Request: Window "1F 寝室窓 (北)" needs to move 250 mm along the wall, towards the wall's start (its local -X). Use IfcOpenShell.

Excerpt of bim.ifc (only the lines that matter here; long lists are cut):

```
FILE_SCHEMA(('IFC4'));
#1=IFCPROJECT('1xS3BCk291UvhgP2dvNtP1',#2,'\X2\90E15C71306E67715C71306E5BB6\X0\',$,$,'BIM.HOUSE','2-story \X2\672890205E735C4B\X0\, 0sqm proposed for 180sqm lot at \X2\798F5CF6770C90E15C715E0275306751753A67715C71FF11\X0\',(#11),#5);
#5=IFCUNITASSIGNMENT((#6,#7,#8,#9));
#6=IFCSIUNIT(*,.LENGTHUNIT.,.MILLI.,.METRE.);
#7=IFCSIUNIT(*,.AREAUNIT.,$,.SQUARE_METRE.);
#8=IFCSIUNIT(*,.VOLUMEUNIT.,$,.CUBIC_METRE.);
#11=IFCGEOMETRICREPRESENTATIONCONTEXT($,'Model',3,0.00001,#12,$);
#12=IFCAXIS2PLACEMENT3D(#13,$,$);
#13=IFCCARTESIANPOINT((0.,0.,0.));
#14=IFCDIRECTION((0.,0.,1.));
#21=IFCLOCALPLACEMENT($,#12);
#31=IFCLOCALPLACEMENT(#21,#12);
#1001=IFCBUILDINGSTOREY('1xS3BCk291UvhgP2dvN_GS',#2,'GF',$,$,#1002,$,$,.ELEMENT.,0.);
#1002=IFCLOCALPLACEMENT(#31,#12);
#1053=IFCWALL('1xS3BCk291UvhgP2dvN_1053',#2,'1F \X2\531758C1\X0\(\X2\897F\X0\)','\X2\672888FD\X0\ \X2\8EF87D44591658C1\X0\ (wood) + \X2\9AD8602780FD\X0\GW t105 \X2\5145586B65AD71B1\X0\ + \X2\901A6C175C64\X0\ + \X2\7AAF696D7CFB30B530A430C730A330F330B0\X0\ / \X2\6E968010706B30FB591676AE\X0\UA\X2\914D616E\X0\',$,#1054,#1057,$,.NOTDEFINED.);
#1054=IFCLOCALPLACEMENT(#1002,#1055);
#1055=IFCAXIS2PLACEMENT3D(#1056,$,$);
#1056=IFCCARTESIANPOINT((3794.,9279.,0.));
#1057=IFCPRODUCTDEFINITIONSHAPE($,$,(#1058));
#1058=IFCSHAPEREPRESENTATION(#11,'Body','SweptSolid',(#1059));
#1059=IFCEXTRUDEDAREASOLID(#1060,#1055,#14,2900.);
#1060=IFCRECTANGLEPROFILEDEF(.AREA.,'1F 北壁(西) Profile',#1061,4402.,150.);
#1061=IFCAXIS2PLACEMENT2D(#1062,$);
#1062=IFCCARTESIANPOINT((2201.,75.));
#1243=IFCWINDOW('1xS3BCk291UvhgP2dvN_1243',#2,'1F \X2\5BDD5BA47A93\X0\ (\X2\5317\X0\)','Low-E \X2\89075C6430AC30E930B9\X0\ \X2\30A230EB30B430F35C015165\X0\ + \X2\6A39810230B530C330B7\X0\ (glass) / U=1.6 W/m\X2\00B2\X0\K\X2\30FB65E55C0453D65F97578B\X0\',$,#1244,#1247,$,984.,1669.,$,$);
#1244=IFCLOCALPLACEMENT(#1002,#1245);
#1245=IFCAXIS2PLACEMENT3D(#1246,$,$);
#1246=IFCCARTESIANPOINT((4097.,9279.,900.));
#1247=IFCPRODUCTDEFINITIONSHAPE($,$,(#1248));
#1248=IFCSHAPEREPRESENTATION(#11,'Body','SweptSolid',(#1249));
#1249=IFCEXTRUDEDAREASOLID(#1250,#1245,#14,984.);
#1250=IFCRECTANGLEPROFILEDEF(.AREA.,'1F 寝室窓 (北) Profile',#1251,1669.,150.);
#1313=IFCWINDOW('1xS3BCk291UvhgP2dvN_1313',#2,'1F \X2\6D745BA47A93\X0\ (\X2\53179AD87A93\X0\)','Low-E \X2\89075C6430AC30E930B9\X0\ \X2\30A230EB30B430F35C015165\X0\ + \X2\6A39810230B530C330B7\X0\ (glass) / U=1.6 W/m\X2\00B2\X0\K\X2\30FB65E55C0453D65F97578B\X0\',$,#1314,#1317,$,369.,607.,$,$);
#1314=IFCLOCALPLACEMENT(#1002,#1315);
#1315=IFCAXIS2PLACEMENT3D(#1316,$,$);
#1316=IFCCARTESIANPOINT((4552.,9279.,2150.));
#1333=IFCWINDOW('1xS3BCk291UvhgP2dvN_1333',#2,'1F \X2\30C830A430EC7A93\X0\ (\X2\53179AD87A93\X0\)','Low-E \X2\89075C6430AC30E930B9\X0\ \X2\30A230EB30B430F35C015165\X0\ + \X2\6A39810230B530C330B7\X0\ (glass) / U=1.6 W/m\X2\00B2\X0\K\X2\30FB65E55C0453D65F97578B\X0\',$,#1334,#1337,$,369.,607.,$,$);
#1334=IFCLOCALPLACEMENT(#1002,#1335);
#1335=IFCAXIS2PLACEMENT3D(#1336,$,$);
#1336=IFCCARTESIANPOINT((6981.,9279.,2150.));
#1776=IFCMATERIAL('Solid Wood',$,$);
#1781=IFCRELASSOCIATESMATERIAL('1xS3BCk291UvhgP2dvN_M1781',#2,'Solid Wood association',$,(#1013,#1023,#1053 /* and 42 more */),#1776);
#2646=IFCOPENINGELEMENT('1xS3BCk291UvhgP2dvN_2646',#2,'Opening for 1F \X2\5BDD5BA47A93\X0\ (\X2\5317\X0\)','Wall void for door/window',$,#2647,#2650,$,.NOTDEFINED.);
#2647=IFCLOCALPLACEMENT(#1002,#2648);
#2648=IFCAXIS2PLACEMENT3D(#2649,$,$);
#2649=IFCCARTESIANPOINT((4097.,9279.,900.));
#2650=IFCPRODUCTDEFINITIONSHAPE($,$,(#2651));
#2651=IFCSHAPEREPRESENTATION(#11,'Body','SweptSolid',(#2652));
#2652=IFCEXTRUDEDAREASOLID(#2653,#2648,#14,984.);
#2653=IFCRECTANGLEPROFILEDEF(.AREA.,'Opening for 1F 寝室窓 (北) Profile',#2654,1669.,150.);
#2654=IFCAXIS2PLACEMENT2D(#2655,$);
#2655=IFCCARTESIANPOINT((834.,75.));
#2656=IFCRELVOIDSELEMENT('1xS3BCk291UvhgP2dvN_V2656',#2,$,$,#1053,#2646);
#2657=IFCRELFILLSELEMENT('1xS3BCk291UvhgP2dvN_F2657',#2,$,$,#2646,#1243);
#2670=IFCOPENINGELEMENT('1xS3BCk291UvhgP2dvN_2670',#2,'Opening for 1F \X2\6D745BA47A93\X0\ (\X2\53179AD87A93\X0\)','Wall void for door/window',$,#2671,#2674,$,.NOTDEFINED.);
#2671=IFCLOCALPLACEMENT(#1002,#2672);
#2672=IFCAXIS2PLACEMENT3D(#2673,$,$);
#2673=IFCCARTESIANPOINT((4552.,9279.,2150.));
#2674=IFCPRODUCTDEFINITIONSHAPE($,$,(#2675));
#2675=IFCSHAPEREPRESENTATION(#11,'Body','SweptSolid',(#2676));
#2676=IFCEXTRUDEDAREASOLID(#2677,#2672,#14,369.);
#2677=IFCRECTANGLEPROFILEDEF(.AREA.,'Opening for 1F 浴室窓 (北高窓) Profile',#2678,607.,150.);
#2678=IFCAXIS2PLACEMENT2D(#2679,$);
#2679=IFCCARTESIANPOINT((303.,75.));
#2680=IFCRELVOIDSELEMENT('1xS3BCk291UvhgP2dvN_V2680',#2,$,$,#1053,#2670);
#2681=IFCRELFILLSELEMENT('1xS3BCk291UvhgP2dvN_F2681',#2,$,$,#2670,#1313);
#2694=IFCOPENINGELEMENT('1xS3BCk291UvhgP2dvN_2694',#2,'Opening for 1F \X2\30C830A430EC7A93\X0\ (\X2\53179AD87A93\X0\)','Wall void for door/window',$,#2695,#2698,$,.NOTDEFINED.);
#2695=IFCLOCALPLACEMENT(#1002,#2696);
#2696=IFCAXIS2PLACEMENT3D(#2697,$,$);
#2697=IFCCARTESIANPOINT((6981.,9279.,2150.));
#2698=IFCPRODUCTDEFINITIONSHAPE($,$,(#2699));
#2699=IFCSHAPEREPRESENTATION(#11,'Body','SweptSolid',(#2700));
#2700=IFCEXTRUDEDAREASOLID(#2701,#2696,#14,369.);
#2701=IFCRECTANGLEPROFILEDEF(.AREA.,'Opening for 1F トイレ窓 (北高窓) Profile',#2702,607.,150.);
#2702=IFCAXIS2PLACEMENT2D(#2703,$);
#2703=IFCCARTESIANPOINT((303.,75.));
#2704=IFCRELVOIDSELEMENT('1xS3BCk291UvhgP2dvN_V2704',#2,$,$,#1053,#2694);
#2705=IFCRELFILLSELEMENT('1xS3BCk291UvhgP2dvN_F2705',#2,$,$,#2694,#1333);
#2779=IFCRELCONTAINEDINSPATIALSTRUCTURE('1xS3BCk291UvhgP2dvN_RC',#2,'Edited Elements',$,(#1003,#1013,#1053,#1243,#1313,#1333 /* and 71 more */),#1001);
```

```python
import ifcopenshell
import ifcopenshell.api.geometry
import ifcopenshell.util.placement
import ifcopenshell.util.unit

model = ifcopenshell.open("bim.ifc")
unit_scale = ifcopenshell.util.unit.calculate_unit_scale(model)

window = model.by_guid("1xS3BCk291UvhgP2dvN_1243")
opening = window.FillsVoids[0].RelatingOpeningElement
wall = opening.VoidsElements[0].RelatingBuildingElement

wall_matrix = ifcopenshell.util.placement.get_local_placement(wall.ObjectPlacement)
shift = wall_matrix[:3, 0] * -0.25 / unit_scale
before = ifcopenshell.util.placement.get_local_placement(window.ObjectPlacement)[:3, 3].copy()

# The window is not placed relative to its opening, so move both.
for product in (opening, window):
    matrix = ifcopenshell.util.placement.get_local_placement(product.ObjectPlacement)
    matrix[:3, 3] += shift
    ifcopenshell.api.geometry.edit_object_placement(model, product=product, matrix=matrix, is_si=False)

after = ifcopenshell.util.placement.get_local_placement(window.ObjectPlacement)[:3, 3]
print("window moved by", (after - before).round(3) + 0.0)

model.write("bim_updated.ifc")
```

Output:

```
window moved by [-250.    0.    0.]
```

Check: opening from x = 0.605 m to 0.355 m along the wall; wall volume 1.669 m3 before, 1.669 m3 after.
